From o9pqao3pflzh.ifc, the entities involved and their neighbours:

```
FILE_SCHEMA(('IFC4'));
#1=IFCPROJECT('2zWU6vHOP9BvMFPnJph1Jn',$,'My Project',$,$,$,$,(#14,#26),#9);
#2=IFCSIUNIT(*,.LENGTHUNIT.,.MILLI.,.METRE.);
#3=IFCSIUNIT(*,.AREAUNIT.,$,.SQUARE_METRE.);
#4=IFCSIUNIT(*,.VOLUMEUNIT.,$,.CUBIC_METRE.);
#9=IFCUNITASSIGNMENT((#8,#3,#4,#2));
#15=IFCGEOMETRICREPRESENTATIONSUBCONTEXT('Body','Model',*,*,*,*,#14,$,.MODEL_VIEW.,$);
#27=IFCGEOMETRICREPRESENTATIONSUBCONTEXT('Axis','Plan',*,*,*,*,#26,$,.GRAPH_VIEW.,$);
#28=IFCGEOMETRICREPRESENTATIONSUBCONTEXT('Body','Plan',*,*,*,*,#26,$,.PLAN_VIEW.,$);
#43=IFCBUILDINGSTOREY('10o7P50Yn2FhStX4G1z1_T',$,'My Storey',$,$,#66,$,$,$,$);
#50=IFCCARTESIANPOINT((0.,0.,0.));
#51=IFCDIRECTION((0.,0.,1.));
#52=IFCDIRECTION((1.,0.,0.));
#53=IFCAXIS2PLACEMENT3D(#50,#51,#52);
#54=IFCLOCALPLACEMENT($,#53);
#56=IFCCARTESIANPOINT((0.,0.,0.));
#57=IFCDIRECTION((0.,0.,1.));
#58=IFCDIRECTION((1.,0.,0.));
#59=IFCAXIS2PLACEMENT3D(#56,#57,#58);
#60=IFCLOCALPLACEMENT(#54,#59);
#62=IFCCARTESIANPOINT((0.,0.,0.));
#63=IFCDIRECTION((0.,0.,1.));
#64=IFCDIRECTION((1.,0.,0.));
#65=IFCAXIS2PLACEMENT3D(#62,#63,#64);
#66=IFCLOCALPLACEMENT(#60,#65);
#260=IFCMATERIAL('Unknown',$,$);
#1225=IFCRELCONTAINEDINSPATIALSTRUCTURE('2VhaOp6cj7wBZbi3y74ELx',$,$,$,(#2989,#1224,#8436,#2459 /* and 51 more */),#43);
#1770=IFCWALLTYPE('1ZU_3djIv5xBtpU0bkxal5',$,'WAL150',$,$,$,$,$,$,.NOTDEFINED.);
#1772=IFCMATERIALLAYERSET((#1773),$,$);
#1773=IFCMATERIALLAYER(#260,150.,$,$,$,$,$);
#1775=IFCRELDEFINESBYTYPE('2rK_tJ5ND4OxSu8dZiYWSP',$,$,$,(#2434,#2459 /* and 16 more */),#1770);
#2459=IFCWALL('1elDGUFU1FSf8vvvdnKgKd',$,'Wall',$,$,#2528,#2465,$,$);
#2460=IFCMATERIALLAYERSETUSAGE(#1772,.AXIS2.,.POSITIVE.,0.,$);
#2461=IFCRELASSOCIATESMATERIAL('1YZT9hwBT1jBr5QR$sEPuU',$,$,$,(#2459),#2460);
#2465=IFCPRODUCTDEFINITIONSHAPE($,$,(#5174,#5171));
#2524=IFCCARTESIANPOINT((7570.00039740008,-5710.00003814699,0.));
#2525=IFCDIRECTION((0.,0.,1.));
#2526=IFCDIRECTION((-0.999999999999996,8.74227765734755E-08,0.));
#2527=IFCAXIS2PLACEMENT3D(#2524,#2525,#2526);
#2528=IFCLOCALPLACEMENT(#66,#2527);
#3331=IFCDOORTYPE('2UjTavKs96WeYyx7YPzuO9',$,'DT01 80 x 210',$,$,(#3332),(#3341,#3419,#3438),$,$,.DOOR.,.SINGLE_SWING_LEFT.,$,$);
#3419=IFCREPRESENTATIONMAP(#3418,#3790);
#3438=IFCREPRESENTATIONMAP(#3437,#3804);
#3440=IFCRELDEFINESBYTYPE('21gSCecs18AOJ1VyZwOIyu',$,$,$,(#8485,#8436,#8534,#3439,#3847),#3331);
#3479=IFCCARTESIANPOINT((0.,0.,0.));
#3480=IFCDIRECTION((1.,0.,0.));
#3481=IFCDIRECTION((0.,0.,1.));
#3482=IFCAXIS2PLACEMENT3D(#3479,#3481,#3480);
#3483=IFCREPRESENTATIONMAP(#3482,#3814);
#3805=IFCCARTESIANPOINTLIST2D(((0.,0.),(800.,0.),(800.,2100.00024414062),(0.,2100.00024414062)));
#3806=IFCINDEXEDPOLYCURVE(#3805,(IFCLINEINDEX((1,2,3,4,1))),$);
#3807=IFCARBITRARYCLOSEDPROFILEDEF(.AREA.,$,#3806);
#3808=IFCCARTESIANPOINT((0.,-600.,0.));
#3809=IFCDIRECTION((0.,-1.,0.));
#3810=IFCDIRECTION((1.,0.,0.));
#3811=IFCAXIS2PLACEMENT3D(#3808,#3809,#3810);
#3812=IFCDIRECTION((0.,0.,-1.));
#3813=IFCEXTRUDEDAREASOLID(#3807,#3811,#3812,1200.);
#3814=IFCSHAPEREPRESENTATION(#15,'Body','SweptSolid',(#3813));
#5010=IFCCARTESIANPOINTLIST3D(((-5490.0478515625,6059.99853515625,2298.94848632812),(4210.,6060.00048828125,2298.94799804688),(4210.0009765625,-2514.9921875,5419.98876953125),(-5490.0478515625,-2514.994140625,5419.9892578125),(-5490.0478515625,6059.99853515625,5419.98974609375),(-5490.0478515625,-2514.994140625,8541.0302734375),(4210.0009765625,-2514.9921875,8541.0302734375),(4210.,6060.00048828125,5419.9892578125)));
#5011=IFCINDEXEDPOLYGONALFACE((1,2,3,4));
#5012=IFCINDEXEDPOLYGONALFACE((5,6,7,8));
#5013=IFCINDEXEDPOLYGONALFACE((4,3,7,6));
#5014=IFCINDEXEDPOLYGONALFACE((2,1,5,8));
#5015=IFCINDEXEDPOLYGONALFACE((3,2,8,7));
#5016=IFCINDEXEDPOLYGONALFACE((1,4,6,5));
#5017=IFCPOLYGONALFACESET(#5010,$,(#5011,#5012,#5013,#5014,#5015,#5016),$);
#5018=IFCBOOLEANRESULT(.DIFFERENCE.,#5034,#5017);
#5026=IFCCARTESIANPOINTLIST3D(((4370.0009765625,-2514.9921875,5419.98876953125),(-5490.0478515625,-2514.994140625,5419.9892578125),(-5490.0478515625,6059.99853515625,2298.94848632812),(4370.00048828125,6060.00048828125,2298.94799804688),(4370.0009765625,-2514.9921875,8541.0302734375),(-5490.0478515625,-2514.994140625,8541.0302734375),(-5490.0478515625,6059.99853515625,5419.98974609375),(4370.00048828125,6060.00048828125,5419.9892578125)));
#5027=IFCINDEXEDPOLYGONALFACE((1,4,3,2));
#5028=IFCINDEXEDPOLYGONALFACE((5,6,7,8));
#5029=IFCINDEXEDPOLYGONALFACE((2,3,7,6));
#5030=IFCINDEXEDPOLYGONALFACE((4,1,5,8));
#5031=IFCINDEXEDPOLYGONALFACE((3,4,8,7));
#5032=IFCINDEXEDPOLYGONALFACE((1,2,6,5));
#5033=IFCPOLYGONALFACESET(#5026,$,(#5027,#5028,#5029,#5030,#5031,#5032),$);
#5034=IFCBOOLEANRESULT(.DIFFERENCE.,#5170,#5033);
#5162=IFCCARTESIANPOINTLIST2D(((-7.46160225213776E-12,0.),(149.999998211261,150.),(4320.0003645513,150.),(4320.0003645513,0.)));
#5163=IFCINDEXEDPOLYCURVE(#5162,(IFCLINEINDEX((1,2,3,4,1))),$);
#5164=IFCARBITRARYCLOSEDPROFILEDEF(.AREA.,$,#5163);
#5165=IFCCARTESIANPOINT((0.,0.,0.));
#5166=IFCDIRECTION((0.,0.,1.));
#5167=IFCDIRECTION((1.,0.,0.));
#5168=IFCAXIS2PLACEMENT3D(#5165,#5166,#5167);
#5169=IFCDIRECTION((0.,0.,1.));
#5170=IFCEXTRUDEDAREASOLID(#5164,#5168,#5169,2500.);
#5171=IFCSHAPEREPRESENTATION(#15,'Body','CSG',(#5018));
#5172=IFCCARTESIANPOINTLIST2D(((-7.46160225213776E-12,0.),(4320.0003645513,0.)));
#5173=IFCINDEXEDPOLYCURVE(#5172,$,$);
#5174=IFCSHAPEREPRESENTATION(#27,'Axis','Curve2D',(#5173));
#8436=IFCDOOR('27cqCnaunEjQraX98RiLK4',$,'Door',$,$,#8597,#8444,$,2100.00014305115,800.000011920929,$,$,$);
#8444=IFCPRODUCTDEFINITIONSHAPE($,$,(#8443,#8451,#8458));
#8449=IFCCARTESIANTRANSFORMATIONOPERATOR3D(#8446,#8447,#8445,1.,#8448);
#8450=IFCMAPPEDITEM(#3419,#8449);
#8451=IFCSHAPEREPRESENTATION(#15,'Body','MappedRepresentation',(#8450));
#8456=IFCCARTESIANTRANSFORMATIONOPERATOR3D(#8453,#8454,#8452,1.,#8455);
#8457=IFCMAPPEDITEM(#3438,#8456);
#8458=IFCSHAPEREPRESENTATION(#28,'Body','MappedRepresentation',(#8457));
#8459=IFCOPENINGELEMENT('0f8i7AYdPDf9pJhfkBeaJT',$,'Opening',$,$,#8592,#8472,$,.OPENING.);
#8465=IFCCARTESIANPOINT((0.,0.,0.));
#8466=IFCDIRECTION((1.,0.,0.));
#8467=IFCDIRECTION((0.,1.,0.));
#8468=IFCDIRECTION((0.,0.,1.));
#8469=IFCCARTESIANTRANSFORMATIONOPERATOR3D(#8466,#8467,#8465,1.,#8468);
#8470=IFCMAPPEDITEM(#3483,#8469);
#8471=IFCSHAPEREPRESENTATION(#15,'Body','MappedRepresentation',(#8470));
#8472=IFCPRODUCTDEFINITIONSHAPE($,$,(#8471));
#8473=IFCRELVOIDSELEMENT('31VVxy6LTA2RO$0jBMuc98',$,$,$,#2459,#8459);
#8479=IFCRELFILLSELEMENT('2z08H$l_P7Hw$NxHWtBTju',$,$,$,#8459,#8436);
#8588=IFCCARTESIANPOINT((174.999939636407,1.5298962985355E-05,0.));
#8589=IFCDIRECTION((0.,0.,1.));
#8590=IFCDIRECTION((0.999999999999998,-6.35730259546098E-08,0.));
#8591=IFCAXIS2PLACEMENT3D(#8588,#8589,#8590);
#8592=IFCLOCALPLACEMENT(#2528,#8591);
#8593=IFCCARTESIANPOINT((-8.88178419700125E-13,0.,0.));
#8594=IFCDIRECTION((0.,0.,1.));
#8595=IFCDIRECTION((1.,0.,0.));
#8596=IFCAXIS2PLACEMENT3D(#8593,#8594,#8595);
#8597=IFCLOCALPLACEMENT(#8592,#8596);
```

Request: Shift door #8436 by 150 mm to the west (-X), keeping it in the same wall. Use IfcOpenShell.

```python
import ifcopenshell
import ifcopenshell.api.geometry
import ifcopenshell.util.placement
import ifcopenshell.util.unit

model = ifcopenshell.open("o9pqao3pflzh.ifc")
unit_scale = ifcopenshell.util.unit.calculate_unit_scale(model)

door = model.by_guid("27cqCnaunEjQraX98RiLK4")
opening = door.FillsVoids[0].RelatingOpeningElement
wall = opening.VoidsElements[0].RelatingBuildingElement

wall_matrix = ifcopenshell.util.placement.get_local_placement(wall.ObjectPlacement)
shift = wall_matrix[:3, 0] * 0.15 / unit_scale
before = ifcopenshell.util.placement.get_local_placement(door.ObjectPlacement)[:3, 3].copy()

# The door is placed relative to its opening, so it follows when the opening moves.
matrix = ifcopenshell.util.placement.get_local_placement(opening.ObjectPlacement)
matrix[:3, 3] += shift
ifcopenshell.api.geometry.edit_object_placement(
    model, product=opening, matrix=matrix, is_si=False, should_transform_children=True
)

after = ifcopenshell.util.placement.get_local_placement(door.ObjectPlacement)[:3, 3]
print("door moved by", (after - before).round(3) + 0.0)

model.write("o9pqao3pflzh_updated.ifc")
```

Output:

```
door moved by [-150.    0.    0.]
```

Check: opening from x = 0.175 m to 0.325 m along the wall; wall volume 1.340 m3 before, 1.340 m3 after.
